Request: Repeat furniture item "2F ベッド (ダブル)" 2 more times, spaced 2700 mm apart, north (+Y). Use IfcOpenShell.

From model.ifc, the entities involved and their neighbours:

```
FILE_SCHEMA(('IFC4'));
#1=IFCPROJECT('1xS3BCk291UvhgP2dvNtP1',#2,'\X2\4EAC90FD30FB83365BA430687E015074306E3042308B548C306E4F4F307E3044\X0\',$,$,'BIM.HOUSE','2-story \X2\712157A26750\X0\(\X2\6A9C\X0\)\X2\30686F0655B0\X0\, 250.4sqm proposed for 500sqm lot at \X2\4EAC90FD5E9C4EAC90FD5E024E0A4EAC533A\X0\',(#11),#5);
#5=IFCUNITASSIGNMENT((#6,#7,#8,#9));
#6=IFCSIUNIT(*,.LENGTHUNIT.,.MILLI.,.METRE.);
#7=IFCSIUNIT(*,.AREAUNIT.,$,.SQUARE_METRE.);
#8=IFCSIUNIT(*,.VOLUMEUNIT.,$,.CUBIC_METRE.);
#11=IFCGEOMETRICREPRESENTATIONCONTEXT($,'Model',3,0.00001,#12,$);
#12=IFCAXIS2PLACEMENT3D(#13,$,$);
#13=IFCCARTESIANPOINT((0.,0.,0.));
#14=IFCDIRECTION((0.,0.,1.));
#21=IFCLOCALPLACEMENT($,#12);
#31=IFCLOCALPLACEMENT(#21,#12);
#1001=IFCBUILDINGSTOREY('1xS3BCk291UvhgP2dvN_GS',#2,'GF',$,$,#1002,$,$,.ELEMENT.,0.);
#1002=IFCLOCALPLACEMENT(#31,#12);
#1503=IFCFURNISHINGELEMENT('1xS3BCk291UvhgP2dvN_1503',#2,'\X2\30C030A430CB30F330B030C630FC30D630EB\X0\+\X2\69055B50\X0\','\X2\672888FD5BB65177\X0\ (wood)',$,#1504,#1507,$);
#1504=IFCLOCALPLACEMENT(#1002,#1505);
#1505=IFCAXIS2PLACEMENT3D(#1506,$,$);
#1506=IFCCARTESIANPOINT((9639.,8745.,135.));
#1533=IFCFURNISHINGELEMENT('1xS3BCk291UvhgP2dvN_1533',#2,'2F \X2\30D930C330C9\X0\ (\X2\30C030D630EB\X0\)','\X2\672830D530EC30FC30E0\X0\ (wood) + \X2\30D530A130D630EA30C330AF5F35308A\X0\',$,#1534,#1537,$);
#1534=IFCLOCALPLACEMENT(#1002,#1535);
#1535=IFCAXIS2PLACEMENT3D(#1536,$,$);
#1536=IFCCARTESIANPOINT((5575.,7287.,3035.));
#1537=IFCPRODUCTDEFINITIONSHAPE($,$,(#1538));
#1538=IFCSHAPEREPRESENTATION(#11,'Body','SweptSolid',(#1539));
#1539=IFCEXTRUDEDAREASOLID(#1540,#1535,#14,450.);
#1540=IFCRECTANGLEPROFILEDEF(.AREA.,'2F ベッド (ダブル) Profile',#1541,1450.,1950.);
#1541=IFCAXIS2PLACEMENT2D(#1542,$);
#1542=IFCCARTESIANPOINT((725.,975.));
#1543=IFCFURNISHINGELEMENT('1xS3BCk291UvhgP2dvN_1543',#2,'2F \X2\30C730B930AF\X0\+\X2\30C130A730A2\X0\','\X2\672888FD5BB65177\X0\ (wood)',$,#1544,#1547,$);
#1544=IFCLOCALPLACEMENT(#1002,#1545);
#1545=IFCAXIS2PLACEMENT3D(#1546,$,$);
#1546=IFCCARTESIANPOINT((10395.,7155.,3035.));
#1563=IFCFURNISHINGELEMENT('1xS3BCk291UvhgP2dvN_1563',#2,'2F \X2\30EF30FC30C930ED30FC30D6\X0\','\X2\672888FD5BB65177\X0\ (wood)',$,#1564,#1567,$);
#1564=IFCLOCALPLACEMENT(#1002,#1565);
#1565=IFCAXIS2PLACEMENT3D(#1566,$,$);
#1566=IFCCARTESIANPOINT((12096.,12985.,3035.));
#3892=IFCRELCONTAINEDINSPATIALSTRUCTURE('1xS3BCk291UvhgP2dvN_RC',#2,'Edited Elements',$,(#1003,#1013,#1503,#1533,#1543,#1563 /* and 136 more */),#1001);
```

```python
import numpy as np
import ifcopenshell
import ifcopenshell.api.geometry
import ifcopenshell.api.root
import ifcopenshell.util.element
import ifcopenshell.util.placement
import ifcopenshell.util.unit

model = ifcopenshell.open("model.ifc")
unit_scale = ifcopenshell.util.unit.calculate_unit_scale(model)


def reuse_history(source, copy):
    """copy_class also copies each property set's owner history, people and application; keep the originals."""
    for rel in copy.IsDefinedBy:
        if rel.is_a("IfcRelDefinesByProperties") and (history := rel.RelatingPropertyDefinition.OwnerHistory):
            rel.RelatingPropertyDefinition.OwnerHistory = source.OwnerHistory
            ifcopenshell.util.element.remove_deep2(model, history)


source = model.by_guid("1xS3BCk291UvhgP2dvN_1533")
base = ifcopenshell.util.placement.get_local_placement(source.ObjectPlacement)
step = np.array([0.0, 1.0, 0.0]) * 2.7 / unit_scale

for i in range(1, 3):
    copy = ifcopenshell.api.root.copy_class(model, product=source)
    copy.Representation = ifcopenshell.util.element.copy_deep(
        model, source.Representation, exclude=["IfcGeometricRepresentationContext", "IfcRepresentationMap"]
    )
    reuse_history(source, copy)
    matrix = base.copy()
    matrix[:3, 3] += i * step
    print("added at", matrix[:3, 3].round(3) + 0.0)
    ifcopenshell.api.geometry.edit_object_placement(model, product=copy, matrix=matrix, is_si=False)

model.write("model_v2.ifc")
```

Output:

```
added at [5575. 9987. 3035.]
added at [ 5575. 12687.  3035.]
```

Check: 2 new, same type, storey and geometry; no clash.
